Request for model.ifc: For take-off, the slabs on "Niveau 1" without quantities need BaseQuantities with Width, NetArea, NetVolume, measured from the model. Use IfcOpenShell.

First a look at what the model holds.

```python
import ifcopenshell
import ifcopenshell.util.element
import ifcopenshell.util.unit

model = ifcopenshell.open("model.ifc")
print(model.schema)
for unit_type in ("LENGTHUNIT", "AREAUNIT", "VOLUMEUNIT"):
    print(unit_type, ifcopenshell.util.unit.calculate_unit_scale(model, unit_type))
storey = next(s for s in model.by_type("IfcBuildingStorey") if s.Name == "Niveau 1")
slabs = [e for e in ifcopenshell.util.element.get_decomposition(storey) if e.is_a("IfcSlab")]
for e in sorted(slabs, key=lambda e: e.id()):
    print(e.id(), e.is_a(), e.Name, list(ifcopenshell.util.element.get_psets(e, qtos_only=True)), sep=" | ")
```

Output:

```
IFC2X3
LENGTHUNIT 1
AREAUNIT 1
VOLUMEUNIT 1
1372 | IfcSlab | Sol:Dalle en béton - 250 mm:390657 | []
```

```python
import ifcopenshell
import ifcopenshell.api.pset
import ifcopenshell.geom
import ifcopenshell.util.element
import ifcopenshell.util.shape
import ifcopenshell.util.unit

model = ifcopenshell.open("model.ifc")
unit_scale = ifcopenshell.util.unit.calculate_unit_scale(model)
area_scale = ifcopenshell.util.unit.calculate_unit_scale(model, "AREAUNIT")
volume_scale = ifcopenshell.util.unit.calculate_unit_scale(model, "VOLUMEUNIT")
settings = ifcopenshell.geom.settings()

storey = next(s for s in model.by_type("IfcBuildingStorey") if s.Name == "Niveau 1")
slabs = [e for e in ifcopenshell.util.element.get_decomposition(storey) if e.is_a("IfcSlab")]

for e in sorted(slabs, key=lambda e: e.id()):
    if ifcopenshell.util.element.get_psets(e, qtos_only=True, should_inherit=False):
        continue
    # Geometry comes back in metres, in the element's own axes.
    shape = ifcopenshell.geom.create_shape(settings, e)
    values = {
        "Width": ifcopenshell.util.shape.get_z(shape.geometry) / unit_scale,
        "NetArea": ifcopenshell.util.shape.get_footprint_area(shape.geometry) / area_scale,
        "NetVolume": ifcopenshell.util.shape.get_volume(shape.geometry) / volume_scale,
    }
    qto = ifcopenshell.api.pset.add_qto(model, product=e, name="BaseQuantities")
    ifcopenshell.api.pset.edit_qto(model, qto=qto, properties=values)
    print(e.id(), {k: round(v, 3) for k, v in values.items()})

model.write("model_edited.ifc")
```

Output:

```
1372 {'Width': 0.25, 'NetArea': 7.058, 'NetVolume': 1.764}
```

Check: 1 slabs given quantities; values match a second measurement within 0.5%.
